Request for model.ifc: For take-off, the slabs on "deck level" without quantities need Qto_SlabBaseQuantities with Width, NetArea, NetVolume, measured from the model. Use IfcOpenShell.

First a look at what the model holds.

```python
import ifcopenshell
import ifcopenshell.util.element
import ifcopenshell.util.unit

model = ifcopenshell.open("model.ifc")
print(model.schema)
for unit_type in ("LENGTHUNIT", "AREAUNIT", "VOLUMEUNIT"):
    print(unit_type, ifcopenshell.util.unit.calculate_unit_scale(model, unit_type))
storey = next(s for s in model.by_type("IfcBuildingStorey") if s.Name == "deck level")
slabs = [e for e in ifcopenshell.util.element.get_decomposition(storey) if e.is_a("IfcSlab")]
for e in sorted(slabs, key=lambda e: e.id()):
    print(e.id(), e.is_a(), e.Name, list(ifcopenshell.util.element.get_psets(e, qtos_only=True)), sep=" | ")
```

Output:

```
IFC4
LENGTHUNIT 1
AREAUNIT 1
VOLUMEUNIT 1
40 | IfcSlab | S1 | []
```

```python
import ifcopenshell
import ifcopenshell.api.pset
import ifcopenshell.geom
import ifcopenshell.util.element
import ifcopenshell.util.shape
import ifcopenshell.util.unit

model = ifcopenshell.open("model.ifc")
unit_scale = ifcopenshell.util.unit.calculate_unit_scale(model)
area_scale = ifcopenshell.util.unit.calculate_unit_scale(model, "AREAUNIT")
volume_scale = ifcopenshell.util.unit.calculate_unit_scale(model, "VOLUMEUNIT")
settings = ifcopenshell.geom.settings()

storey = next(s for s in model.by_type("IfcBuildingStorey") if s.Name == "deck level")
slabs = [e for e in ifcopenshell.util.element.get_decomposition(storey) if e.is_a("IfcSlab")]

for e in sorted(slabs, key=lambda e: e.id()):
    if ifcopenshell.util.element.get_psets(e, qtos_only=True, should_inherit=False):
        continue
    # Geometry comes back in metres, in the element's own axes.
    shape = ifcopenshell.geom.create_shape(settings, e)
    values = {
        "Width": ifcopenshell.util.shape.get_z(shape.geometry) / unit_scale,
        "NetArea": ifcopenshell.util.shape.get_footprint_area(shape.geometry) / area_scale,
        "NetVolume": ifcopenshell.util.shape.get_volume(shape.geometry) / volume_scale,
    }
    qto = ifcopenshell.api.pset.add_qto(model, product=e, name="Qto_SlabBaseQuantities")
    ifcopenshell.api.pset.edit_qto(model, qto=qto, properties=values)
    print(e.id(), {k: round(v, 3) for k, v in values.items()})

model.write("model_edited.ifc")
```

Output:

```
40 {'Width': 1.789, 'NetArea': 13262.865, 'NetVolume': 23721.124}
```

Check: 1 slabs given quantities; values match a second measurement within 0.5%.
